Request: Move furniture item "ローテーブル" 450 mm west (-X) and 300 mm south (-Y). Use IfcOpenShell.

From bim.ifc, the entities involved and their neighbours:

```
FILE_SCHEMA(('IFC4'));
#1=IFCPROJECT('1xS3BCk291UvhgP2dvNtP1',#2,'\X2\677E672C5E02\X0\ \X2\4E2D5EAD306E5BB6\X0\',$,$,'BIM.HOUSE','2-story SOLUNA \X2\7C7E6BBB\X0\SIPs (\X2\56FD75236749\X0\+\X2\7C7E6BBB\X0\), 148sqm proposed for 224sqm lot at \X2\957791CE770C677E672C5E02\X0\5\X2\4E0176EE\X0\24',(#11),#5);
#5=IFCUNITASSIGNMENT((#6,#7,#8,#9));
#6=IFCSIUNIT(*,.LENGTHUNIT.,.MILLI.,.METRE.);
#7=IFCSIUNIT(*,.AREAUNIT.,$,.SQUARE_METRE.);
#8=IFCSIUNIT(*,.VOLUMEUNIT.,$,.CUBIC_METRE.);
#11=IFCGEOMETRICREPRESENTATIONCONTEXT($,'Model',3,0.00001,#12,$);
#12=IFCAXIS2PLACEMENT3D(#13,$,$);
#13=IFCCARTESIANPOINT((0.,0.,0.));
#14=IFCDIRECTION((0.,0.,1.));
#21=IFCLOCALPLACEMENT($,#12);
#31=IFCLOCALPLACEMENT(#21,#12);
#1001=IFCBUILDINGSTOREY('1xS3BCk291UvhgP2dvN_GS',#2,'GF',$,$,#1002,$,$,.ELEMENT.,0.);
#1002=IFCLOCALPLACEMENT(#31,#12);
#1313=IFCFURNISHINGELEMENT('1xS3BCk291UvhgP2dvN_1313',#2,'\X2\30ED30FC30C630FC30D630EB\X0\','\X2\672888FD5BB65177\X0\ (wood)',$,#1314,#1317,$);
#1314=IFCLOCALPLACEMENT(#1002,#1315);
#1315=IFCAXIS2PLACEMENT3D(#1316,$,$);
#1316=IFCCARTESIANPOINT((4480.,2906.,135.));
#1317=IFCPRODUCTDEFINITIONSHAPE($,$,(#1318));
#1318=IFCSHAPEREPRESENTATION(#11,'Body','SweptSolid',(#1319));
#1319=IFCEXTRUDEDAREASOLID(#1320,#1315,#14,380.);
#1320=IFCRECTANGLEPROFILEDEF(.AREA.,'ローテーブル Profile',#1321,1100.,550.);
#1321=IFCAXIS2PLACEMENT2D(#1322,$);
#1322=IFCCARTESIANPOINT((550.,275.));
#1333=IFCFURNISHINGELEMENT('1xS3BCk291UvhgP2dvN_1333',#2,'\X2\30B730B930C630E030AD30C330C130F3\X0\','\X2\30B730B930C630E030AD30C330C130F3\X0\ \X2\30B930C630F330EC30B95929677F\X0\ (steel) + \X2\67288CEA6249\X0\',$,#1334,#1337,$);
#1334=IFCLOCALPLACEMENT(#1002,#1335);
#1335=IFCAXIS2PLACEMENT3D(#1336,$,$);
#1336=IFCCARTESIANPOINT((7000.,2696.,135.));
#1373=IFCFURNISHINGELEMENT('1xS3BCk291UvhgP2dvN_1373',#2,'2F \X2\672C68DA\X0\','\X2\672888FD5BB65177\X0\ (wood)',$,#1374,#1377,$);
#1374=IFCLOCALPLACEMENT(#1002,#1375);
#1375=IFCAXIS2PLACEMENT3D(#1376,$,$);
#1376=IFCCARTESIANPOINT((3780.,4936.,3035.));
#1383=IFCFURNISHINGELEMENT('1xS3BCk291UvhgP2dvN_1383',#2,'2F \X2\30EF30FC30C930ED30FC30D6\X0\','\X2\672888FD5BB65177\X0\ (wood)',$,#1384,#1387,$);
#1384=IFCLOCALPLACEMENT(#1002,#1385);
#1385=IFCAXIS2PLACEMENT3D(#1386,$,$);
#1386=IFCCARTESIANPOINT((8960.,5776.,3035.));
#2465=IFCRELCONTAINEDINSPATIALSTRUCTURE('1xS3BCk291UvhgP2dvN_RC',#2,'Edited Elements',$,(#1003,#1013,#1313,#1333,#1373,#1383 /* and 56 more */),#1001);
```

```python
import ifcopenshell
import ifcopenshell.api.geometry
import ifcopenshell.util.placement
import ifcopenshell.util.unit

model = ifcopenshell.open("bim.ifc")
unit_scale = ifcopenshell.util.unit.calculate_unit_scale(model)

item = model.by_guid("1xS3BCk291UvhgP2dvN_1313")
matrix = ifcopenshell.util.placement.get_local_placement(item.ObjectPlacement)
matrix[0, 3] -= 0.45 / unit_scale
matrix[1, 3] -= 0.3 / unit_scale
ifcopenshell.api.geometry.edit_object_placement(model, product=item, matrix=matrix, is_si=False)

print(ifcopenshell.util.placement.get_local_placement(item.ObjectPlacement).round(3) + 0.0)

model.write("bim_updated.ifc")
```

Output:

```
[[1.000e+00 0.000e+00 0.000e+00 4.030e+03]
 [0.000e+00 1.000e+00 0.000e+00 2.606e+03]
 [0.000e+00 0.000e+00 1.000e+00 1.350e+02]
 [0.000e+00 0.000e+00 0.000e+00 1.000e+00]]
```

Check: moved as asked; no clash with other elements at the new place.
